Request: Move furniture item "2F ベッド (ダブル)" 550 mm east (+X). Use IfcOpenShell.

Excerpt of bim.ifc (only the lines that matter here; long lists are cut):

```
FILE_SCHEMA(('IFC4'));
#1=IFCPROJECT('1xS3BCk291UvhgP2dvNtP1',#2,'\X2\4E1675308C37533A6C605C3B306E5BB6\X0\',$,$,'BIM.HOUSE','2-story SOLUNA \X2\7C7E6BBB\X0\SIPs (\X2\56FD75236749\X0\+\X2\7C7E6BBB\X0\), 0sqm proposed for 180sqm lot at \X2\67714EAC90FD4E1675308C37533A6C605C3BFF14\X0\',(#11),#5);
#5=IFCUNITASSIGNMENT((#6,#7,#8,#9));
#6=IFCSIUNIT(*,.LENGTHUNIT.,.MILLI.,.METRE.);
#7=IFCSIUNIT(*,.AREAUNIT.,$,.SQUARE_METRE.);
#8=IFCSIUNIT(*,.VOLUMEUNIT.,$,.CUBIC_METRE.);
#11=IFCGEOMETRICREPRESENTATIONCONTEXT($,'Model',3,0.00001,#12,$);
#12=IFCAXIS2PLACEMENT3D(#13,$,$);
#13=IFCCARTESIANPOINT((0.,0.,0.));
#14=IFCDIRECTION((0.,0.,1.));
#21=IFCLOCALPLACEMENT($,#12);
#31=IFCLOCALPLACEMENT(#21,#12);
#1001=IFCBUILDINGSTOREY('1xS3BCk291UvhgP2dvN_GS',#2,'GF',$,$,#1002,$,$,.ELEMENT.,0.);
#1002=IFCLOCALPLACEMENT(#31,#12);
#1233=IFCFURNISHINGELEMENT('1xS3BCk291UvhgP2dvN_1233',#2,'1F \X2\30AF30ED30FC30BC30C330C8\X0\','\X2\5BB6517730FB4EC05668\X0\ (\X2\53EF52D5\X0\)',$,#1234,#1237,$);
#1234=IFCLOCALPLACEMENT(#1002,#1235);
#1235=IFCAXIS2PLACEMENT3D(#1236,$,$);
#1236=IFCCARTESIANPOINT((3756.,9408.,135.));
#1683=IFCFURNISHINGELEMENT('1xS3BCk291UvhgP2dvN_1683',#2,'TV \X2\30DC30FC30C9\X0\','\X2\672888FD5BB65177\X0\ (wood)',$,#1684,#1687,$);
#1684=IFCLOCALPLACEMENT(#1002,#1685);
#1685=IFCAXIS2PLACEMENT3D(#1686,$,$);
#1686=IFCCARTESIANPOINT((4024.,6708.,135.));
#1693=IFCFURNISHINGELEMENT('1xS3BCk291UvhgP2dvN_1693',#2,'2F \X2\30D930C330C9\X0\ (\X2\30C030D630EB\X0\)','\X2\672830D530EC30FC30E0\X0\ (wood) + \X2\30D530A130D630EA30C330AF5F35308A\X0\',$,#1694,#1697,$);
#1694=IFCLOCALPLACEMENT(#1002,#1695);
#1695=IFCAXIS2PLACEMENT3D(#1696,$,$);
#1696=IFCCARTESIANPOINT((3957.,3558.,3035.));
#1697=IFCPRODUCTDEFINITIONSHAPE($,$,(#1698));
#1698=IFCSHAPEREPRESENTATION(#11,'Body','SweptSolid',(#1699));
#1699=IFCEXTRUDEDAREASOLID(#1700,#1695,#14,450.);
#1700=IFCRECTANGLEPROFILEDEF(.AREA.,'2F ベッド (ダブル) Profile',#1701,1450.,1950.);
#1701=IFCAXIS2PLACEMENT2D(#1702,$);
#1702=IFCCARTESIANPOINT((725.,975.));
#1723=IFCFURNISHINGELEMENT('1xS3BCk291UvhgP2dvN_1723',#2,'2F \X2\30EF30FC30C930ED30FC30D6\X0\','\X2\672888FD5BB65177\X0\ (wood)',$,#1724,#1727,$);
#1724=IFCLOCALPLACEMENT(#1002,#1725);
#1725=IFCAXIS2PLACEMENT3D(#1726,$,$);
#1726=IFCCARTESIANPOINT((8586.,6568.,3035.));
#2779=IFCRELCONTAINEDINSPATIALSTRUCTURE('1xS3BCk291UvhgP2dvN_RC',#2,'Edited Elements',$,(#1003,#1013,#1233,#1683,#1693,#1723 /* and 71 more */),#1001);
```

```python
import ifcopenshell
import ifcopenshell.api.geometry
import ifcopenshell.util.placement

model = ifcopenshell.open("bim.ifc")

item = model.by_guid("1xS3BCk291UvhgP2dvN_1693")
matrix = ifcopenshell.util.placement.get_local_placement(item.ObjectPlacement)
matrix[0, 3] += 550.0
ifcopenshell.api.geometry.edit_object_placement(model, product=item, matrix=matrix, is_si=False)

print(ifcopenshell.util.placement.get_local_placement(item.ObjectPlacement).round(3) + 0.0)

model.write("bim_updated.ifc")
```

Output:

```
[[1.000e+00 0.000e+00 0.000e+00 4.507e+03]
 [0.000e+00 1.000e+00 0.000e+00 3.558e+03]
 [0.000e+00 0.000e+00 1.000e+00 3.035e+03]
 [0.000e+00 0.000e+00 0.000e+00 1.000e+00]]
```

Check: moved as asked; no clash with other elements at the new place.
